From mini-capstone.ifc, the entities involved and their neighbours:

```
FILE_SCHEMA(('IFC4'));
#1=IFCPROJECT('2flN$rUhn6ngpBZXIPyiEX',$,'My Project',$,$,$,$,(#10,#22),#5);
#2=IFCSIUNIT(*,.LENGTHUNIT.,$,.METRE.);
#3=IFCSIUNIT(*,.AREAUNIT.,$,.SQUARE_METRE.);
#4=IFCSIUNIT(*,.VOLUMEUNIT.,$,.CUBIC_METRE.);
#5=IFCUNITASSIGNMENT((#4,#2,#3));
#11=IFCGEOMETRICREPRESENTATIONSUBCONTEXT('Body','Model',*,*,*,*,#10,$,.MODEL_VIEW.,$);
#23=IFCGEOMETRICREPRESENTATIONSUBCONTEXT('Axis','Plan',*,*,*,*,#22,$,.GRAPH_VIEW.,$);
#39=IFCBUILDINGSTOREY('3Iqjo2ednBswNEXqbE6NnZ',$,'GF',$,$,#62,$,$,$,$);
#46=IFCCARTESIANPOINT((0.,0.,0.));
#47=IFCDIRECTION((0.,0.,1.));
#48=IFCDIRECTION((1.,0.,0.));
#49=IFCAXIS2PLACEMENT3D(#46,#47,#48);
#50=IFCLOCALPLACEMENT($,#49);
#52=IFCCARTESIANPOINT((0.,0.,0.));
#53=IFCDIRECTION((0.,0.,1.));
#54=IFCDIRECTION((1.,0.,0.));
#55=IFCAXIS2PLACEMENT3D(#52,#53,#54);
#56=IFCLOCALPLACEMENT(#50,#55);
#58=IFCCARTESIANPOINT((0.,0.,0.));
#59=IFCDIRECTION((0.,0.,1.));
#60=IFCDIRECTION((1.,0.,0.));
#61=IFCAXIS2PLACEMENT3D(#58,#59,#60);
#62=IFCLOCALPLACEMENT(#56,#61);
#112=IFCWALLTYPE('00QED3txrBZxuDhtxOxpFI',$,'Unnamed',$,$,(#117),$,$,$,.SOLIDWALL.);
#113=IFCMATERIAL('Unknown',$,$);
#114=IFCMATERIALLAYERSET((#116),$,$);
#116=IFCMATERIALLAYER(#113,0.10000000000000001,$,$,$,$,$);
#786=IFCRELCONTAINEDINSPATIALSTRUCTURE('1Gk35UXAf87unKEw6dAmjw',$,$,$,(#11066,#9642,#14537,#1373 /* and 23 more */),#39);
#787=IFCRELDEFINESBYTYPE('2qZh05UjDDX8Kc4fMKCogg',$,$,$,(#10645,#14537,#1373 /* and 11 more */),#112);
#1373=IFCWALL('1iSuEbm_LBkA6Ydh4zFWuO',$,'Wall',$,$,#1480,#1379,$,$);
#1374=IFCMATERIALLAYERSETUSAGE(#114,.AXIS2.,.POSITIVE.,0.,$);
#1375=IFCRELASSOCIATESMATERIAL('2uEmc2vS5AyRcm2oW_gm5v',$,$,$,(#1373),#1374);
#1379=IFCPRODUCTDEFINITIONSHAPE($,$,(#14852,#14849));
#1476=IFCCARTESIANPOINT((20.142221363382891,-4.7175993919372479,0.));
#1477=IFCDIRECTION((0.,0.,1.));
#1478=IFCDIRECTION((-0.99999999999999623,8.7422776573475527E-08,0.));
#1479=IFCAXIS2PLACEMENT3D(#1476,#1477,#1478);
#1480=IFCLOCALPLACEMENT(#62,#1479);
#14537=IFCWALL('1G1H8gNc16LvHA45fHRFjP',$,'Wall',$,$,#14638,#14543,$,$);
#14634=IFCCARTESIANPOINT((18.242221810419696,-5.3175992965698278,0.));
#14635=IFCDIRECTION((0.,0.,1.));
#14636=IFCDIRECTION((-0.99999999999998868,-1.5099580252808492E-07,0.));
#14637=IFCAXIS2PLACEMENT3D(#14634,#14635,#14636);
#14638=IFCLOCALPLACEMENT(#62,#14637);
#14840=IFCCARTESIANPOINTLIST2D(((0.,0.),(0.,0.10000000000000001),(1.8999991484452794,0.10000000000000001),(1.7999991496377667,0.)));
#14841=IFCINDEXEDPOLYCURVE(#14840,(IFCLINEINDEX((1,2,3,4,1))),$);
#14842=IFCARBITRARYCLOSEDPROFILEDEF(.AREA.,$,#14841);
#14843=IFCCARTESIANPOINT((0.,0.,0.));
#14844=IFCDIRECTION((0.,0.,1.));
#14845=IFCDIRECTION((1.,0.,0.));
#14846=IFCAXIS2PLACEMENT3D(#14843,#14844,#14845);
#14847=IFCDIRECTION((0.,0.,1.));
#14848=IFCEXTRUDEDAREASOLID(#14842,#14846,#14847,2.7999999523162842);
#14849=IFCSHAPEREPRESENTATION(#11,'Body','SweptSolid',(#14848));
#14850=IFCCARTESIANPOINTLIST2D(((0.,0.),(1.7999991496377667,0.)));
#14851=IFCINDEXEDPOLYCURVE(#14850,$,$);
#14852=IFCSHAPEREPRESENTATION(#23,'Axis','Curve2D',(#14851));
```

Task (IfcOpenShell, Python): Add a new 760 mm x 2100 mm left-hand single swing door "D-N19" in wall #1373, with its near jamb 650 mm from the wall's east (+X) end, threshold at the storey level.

```python
import numpy as np
import ifcopenshell
import ifcopenshell.api.feature
import ifcopenshell.api.geometry
import ifcopenshell.api.root
import ifcopenshell.api.spatial
import ifcopenshell.geom
import ifcopenshell.util.element
import ifcopenshell.util.placement
import ifcopenshell.util.representation
import ifcopenshell.util.shape
import ifcopenshell.util.unit

model = ifcopenshell.open("mini-capstone.ifc")
unit_scale = ifcopenshell.util.unit.calculate_unit_scale(model)
settings = ifcopenshell.geom.settings()


def volume(element):
    """Net volume in cubic metres, openings subtracted."""
    shape = ifcopenshell.geom.create_shape(settings, element)
    return ifcopenshell.util.shape.get_volume(shape.geometry)


wall = model.by_guid("1iSuEbm_LBkA6Ydh4zFWuO")
storey = ifcopenshell.util.element.get_container(wall, ifc_class="IfcBuildingStorey")
context = ifcopenshell.util.representation.get_context(model, "Model", "Body", "MODEL_VIEW")
before = volume(wall)

width, height, from_end, sill = 0.76, 2.1, 0.65, 0.0  # metres

# The wall runs along its own X axis, and the end named is its -X end.
wall_shape = ifcopenshell.geom.create_shape(settings, wall)
x, y, z = ifcopenshell.util.shape.get_vertices(wall_shape.geometry).T
start = x.min() + from_end
face, thickness = float(y.min()), float(y.max() - y.min())
wall_matrix = ifcopenshell.util.placement.get_local_placement(wall.ObjectPlacement)
level = ifcopenshell.util.placement.get_local_placement(storey.ObjectPlacement)[2, 3]


def in_wall(x, y):
    """Placement at x, y metres in the wall's axes, at sill height."""
    matrix = wall_matrix.copy()
    matrix[:, 3] = wall_matrix @ np.array([x / unit_scale, y / unit_scale, 0.0, 1.0])
    matrix[2, 3] = level + sill / unit_scale
    return matrix


# Opening: a box that overshoots both wall faces by 50 mm.
opening = ifcopenshell.api.root.create_entity(model, ifc_class="IfcOpeningElement", predefined_type="OPENING")
box = ifcopenshell.api.geometry.add_wall_representation(
    model, context=context, length=width, height=height, thickness=thickness + 0.1
)
ifcopenshell.api.geometry.assign_representation(model, product=opening, representation=box)
ifcopenshell.api.geometry.edit_object_placement(model, product=opening, matrix=in_wall(start, face - 0.05), is_si=False)
ifcopenshell.api.feature.add_feature(model, feature=opening, element=wall)

door = ifcopenshell.api.root.create_entity(model, ifc_class="IfcDoor", name="D-N19", predefined_type="DOOR")
door.OverallWidth, door.OverallHeight = width / unit_scale, height / unit_scale
door.OperationType = "SINGLE_SWING_LEFT"
body = ifcopenshell.api.geometry.add_door_representation(
    model,
    context=context,
    overall_width=door.OverallWidth,
    overall_height=door.OverallHeight,
    operation_type="SINGLE_SWING_LEFT",
    lining_properties={"LiningDepth": thickness / unit_scale, "ThresholdDepth": thickness / unit_scale},
)
ifcopenshell.api.geometry.assign_representation(model, product=door, representation=body)
ifcopenshell.api.spatial.assign_container(model, products=[door], relating_structure=storey)
ifcopenshell.api.feature.add_filling(model, opening=opening, element=door)

# The lining spans the wall, so the door starts at the wall face.
ifcopenshell.api.geometry.edit_object_placement(model, product=door, matrix=in_wall(start, face), is_si=False)

after = volume(wall)

print(f"wall volume {before:.3f} -> {after:.3f} m3")

model.write("mini-capstone-out.ifc")
```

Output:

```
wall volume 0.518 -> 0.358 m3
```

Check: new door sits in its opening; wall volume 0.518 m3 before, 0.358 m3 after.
